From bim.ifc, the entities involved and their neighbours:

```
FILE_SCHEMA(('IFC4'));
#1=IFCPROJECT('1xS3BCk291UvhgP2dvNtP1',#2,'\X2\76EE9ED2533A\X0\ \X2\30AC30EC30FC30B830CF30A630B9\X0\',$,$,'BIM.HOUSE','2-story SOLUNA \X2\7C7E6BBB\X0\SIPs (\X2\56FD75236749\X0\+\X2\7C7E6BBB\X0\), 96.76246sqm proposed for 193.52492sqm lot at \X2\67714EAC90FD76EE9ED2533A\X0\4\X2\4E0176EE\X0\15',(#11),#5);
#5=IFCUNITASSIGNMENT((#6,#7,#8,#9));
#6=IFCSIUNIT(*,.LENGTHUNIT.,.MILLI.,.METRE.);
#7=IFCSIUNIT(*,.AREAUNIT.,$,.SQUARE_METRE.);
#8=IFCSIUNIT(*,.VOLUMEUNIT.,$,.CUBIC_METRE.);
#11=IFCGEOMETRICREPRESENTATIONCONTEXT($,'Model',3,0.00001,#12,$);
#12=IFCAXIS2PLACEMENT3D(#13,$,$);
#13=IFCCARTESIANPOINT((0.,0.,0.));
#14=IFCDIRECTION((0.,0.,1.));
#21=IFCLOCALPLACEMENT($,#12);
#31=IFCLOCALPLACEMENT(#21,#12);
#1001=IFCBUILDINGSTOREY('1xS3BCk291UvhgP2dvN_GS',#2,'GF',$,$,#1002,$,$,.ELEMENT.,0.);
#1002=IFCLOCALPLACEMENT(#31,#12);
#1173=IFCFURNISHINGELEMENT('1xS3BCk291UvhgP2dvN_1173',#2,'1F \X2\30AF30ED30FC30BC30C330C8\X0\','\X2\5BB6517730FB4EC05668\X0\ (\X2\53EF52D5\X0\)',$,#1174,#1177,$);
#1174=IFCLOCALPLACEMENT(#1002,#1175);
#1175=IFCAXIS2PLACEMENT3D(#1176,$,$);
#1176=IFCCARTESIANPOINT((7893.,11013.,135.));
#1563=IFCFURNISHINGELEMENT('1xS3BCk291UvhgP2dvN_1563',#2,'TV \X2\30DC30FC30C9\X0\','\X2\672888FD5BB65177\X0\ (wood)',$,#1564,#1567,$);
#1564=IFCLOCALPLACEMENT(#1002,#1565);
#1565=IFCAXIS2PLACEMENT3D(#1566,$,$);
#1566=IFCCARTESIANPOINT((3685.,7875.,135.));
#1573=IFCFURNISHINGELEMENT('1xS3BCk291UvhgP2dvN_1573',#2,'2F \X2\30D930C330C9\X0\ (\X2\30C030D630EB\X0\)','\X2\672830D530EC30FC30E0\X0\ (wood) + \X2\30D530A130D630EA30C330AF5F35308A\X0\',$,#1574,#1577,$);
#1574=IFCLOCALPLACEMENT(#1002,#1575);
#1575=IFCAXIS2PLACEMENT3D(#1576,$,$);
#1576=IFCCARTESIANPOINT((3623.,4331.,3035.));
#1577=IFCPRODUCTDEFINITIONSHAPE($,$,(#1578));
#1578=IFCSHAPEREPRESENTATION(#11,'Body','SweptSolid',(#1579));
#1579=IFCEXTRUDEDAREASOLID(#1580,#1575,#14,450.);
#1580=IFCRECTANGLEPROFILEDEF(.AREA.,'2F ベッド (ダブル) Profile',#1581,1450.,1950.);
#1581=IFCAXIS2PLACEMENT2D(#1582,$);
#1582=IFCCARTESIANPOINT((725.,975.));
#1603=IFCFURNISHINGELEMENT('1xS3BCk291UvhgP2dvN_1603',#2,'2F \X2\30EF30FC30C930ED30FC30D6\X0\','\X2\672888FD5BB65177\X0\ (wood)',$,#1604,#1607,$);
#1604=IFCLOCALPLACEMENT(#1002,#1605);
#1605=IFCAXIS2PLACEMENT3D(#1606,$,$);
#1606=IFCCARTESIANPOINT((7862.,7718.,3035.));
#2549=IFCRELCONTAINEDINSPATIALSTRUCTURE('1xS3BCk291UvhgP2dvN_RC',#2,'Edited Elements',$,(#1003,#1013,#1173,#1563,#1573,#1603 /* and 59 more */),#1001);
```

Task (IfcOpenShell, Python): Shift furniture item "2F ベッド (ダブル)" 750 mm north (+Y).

```python
import ifcopenshell
import ifcopenshell.api.geometry
import ifcopenshell.util.placement

model = ifcopenshell.open("bim.ifc")

item = model.by_guid("1xS3BCk291UvhgP2dvN_1573")
matrix = ifcopenshell.util.placement.get_local_placement(item.ObjectPlacement)
matrix[1, 3] += 750.0
ifcopenshell.api.geometry.edit_object_placement(model, product=item, matrix=matrix, is_si=False)

print(ifcopenshell.util.placement.get_local_placement(item.ObjectPlacement).round(3) + 0.0)

model.write("bim_updated.ifc")
```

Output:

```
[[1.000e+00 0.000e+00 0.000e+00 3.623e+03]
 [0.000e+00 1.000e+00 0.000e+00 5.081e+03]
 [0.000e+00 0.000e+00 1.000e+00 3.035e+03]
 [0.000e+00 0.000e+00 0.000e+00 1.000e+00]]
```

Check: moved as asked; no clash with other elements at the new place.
